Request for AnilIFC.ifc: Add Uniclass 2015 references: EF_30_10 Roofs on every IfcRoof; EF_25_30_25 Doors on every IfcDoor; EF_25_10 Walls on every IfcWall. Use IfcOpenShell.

First a look at what the model holds.

```python
import ifcopenshell

model = ifcopenshell.open("AnilIFC.ifc")
print(model.schema)
print("classifications:", [c.Name for c in model.by_type("IfcClassification")])
for ifc_class in ("IfcDoor", "IfcRoof", "IfcStair", "IfcWall", "IfcWindow"):
    print(ifc_class, len(model.by_type(ifc_class)))
```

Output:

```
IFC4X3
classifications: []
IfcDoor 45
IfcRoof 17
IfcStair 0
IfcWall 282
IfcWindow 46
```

```python
import ifcopenshell
import ifcopenshell.api.classification

model = ifcopenshell.open("AnilIFC.ifc")

system = ifcopenshell.api.classification.add_classification(model, classification="Uniclass 2015")

codes = {
    "IfcRoof": ("EF_30_10", "Roofs"),
    "IfcDoor": ("EF_25_30_25", "Doors"),
    "IfcWall": ("EF_25_10", "Walls"),
}
for ifc_class, (code, name) in codes.items():
    products = model.by_type(ifc_class)
    ifcopenshell.api.classification.add_reference(
        model, products=products, classification=system, identification=code, name=name
    )
    print(code, len(products))

model.write("AnilIFC-out.ifc")
```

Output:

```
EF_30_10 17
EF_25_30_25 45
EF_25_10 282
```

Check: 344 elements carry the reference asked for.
